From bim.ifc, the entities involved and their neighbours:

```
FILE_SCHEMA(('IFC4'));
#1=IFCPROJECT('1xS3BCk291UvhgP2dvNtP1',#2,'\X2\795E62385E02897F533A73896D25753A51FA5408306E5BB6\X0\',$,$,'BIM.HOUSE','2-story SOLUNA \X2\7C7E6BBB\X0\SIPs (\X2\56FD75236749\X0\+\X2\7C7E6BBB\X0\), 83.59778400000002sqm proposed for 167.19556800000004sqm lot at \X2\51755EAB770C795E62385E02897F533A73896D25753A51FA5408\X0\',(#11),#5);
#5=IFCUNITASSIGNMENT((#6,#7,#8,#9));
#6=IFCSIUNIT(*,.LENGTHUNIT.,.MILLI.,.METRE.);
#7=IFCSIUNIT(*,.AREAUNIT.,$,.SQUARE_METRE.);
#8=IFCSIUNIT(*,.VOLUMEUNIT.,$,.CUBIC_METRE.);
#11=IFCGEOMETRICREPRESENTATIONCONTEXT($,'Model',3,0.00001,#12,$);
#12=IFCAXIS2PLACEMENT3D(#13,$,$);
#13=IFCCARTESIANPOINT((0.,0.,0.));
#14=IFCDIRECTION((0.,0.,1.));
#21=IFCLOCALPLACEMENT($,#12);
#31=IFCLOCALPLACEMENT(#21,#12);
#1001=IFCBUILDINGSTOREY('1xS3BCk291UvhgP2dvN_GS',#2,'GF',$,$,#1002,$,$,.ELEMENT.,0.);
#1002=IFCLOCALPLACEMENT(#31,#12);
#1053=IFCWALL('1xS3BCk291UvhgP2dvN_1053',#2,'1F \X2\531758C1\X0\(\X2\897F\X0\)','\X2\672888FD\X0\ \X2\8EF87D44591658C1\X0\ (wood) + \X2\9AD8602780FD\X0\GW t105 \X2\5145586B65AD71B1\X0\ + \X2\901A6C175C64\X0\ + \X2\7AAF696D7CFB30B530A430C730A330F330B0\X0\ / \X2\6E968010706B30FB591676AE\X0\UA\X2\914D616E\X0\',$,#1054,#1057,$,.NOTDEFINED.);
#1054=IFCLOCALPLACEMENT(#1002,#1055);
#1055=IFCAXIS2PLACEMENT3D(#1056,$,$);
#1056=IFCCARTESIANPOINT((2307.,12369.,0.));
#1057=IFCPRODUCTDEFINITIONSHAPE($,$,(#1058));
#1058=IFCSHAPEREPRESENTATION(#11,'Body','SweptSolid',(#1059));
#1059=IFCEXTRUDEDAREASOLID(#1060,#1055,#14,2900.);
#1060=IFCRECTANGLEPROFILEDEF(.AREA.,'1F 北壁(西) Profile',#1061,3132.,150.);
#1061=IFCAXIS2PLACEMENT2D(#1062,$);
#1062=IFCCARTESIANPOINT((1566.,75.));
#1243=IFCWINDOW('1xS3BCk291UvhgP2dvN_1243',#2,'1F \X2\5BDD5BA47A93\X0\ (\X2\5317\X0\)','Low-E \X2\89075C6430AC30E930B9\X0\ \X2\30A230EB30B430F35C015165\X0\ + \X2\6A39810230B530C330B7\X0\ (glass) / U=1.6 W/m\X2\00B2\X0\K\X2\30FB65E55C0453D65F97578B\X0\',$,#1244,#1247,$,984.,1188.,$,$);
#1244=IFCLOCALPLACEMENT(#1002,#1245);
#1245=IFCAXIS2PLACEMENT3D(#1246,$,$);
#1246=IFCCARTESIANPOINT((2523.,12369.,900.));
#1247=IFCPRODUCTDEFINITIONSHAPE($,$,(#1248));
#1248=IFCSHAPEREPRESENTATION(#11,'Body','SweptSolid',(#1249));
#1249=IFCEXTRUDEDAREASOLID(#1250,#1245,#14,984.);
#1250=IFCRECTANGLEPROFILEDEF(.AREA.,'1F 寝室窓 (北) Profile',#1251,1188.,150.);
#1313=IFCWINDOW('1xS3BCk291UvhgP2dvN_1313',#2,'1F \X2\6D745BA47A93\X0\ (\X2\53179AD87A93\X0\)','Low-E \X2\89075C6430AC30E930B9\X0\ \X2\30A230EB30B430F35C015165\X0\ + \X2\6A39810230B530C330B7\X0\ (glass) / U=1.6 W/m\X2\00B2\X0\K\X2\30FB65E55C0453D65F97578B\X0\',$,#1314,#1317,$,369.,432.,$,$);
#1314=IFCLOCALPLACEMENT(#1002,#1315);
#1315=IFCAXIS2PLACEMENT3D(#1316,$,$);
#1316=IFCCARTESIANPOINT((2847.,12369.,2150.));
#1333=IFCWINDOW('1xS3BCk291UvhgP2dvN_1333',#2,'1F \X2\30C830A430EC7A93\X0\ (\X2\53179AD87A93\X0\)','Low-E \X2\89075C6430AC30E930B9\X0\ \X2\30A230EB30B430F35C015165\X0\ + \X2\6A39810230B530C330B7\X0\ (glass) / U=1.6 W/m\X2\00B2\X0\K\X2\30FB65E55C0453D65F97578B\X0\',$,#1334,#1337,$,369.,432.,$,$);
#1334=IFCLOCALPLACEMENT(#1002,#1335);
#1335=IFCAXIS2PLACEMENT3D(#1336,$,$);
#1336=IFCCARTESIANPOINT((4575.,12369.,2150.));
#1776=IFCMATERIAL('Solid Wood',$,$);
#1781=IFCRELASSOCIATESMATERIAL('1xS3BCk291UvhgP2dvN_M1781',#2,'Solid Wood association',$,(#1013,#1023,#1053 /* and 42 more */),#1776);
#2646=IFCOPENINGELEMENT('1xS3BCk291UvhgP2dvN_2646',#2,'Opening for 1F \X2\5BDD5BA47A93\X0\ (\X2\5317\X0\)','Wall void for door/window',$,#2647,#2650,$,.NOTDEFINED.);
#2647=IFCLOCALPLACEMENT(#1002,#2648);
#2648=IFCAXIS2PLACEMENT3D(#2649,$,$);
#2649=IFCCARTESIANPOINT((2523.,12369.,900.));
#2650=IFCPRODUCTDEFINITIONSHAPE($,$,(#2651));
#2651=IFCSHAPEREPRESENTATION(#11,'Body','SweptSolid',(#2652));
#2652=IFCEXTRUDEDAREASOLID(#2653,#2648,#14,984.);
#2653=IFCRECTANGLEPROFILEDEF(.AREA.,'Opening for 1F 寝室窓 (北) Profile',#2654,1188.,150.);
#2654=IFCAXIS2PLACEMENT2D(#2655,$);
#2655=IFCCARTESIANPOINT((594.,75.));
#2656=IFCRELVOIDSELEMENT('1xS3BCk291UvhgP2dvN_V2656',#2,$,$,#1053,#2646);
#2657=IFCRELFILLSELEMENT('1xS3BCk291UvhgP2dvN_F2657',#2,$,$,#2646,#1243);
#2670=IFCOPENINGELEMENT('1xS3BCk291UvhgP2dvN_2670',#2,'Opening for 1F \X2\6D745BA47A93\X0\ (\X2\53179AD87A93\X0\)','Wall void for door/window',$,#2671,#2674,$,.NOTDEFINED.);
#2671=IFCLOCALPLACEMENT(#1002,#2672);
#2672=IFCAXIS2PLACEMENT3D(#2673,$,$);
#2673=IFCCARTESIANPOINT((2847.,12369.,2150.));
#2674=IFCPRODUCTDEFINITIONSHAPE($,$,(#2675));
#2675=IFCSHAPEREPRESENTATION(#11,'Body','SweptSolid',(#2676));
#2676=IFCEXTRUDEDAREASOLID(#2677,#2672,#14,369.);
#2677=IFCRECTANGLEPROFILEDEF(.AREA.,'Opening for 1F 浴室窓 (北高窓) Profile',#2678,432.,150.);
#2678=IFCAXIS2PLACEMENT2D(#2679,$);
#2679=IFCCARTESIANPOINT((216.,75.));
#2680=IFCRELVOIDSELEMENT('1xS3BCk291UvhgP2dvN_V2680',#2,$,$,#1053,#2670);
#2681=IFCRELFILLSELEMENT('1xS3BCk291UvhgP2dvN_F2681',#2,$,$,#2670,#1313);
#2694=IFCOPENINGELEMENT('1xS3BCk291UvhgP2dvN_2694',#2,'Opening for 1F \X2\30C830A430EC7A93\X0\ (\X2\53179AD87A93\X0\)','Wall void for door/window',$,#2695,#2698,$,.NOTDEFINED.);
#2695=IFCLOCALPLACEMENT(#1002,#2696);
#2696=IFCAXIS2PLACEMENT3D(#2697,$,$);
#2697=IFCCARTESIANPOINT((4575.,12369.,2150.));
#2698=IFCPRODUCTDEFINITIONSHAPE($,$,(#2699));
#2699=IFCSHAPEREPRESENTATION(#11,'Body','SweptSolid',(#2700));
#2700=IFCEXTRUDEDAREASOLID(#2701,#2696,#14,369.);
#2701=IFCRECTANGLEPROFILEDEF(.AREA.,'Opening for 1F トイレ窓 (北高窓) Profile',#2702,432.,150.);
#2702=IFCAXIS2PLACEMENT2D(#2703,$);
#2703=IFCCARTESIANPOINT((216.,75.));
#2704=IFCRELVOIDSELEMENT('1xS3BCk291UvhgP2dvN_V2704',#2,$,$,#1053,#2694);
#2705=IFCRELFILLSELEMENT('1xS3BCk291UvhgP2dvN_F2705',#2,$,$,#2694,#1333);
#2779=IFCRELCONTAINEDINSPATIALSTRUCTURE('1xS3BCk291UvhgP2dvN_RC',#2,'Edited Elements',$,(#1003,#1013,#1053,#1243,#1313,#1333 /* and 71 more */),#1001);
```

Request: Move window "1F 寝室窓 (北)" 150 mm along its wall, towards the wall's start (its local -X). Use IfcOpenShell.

```python
import ifcopenshell
import ifcopenshell.api.geometry
import ifcopenshell.util.placement

model = ifcopenshell.open("bim.ifc")

window = model.by_id(1243)
opening = window.FillsVoids[0].RelatingOpeningElement
wall = opening.VoidsElements[0].RelatingBuildingElement

wall_matrix = ifcopenshell.util.placement.get_local_placement(wall.ObjectPlacement)
shift = wall_matrix[:3, 0] * -150.0
before = ifcopenshell.util.placement.get_local_placement(window.ObjectPlacement)[:3, 3].copy()

# The window is not placed relative to its opening, so move both.
for product in (opening, window):
    matrix = ifcopenshell.util.placement.get_local_placement(product.ObjectPlacement)
    matrix[:3, 3] += shift
    ifcopenshell.api.geometry.edit_object_placement(model, product=product, matrix=matrix, is_si=False)

after = ifcopenshell.util.placement.get_local_placement(window.ObjectPlacement)[:3, 3]
print("window moved by", (after - before).round(3) + 0.0)

model.write("bim_v2.ifc")
```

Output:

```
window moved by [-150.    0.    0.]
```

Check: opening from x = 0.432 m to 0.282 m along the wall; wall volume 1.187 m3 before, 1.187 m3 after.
